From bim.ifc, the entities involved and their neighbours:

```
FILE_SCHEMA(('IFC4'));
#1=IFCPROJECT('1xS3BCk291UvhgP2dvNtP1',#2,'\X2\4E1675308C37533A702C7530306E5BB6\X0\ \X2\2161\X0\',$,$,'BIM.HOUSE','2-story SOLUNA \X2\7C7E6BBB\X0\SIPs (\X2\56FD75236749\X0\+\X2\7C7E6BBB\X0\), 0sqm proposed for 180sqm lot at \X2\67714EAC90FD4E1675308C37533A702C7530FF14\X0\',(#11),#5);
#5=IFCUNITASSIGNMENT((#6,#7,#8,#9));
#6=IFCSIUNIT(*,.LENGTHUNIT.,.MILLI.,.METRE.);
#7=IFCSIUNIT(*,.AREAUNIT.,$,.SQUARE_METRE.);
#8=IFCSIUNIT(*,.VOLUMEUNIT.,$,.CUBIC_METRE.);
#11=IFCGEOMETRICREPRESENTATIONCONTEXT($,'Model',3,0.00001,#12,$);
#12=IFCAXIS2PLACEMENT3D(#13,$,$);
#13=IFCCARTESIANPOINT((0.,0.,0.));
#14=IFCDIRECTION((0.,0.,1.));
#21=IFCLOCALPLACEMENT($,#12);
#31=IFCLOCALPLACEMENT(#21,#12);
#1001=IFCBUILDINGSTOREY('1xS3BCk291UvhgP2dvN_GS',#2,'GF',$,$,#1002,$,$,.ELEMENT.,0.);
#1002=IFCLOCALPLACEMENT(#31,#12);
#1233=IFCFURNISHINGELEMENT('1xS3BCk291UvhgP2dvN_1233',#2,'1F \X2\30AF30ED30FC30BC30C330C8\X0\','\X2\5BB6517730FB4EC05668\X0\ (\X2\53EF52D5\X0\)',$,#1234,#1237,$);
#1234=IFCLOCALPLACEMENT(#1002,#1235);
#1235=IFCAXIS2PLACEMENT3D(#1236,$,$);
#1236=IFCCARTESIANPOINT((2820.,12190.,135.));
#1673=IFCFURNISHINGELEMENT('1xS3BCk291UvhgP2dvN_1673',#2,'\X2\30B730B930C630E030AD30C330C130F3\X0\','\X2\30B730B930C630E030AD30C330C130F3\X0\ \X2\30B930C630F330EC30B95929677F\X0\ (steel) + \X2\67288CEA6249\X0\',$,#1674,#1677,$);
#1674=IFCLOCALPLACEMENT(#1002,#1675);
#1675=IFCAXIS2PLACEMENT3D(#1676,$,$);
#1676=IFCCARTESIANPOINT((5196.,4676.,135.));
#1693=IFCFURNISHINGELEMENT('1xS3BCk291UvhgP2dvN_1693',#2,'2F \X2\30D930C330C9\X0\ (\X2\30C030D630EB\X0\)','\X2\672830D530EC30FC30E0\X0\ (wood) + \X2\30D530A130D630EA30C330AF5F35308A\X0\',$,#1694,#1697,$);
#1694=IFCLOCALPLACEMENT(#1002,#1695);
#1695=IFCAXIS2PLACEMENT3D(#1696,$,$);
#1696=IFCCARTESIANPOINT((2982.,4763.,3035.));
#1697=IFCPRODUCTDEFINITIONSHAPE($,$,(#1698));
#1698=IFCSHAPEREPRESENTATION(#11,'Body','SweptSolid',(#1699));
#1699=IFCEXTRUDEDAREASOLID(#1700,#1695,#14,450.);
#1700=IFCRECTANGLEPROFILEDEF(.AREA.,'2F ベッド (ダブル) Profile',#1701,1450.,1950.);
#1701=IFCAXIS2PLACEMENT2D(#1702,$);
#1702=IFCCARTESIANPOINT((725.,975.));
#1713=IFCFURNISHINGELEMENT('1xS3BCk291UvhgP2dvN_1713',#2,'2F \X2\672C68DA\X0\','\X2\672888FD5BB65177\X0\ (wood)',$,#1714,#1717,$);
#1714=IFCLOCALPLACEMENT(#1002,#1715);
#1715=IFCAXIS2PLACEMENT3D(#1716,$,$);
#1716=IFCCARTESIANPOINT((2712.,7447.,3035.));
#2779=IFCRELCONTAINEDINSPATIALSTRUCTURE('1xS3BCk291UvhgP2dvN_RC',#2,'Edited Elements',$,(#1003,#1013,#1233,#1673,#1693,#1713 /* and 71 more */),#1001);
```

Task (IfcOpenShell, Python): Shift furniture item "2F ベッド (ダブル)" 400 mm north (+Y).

```python
import ifcopenshell
import ifcopenshell.api.geometry
import ifcopenshell.util.placement

model = ifcopenshell.open("bim.ifc")

item = model.by_guid("1xS3BCk291UvhgP2dvN_1693")
matrix = ifcopenshell.util.placement.get_local_placement(item.ObjectPlacement)
matrix[1, 3] += 400.0
ifcopenshell.api.geometry.edit_object_placement(model, product=item, matrix=matrix, is_si=False)

print(ifcopenshell.util.placement.get_local_placement(item.ObjectPlacement).round(3) + 0.0)

model.write("bim_edited.ifc")
```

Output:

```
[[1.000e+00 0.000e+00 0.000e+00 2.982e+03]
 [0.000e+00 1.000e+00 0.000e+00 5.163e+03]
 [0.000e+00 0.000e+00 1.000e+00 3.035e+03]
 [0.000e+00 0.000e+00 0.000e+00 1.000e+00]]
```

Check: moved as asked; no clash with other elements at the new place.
